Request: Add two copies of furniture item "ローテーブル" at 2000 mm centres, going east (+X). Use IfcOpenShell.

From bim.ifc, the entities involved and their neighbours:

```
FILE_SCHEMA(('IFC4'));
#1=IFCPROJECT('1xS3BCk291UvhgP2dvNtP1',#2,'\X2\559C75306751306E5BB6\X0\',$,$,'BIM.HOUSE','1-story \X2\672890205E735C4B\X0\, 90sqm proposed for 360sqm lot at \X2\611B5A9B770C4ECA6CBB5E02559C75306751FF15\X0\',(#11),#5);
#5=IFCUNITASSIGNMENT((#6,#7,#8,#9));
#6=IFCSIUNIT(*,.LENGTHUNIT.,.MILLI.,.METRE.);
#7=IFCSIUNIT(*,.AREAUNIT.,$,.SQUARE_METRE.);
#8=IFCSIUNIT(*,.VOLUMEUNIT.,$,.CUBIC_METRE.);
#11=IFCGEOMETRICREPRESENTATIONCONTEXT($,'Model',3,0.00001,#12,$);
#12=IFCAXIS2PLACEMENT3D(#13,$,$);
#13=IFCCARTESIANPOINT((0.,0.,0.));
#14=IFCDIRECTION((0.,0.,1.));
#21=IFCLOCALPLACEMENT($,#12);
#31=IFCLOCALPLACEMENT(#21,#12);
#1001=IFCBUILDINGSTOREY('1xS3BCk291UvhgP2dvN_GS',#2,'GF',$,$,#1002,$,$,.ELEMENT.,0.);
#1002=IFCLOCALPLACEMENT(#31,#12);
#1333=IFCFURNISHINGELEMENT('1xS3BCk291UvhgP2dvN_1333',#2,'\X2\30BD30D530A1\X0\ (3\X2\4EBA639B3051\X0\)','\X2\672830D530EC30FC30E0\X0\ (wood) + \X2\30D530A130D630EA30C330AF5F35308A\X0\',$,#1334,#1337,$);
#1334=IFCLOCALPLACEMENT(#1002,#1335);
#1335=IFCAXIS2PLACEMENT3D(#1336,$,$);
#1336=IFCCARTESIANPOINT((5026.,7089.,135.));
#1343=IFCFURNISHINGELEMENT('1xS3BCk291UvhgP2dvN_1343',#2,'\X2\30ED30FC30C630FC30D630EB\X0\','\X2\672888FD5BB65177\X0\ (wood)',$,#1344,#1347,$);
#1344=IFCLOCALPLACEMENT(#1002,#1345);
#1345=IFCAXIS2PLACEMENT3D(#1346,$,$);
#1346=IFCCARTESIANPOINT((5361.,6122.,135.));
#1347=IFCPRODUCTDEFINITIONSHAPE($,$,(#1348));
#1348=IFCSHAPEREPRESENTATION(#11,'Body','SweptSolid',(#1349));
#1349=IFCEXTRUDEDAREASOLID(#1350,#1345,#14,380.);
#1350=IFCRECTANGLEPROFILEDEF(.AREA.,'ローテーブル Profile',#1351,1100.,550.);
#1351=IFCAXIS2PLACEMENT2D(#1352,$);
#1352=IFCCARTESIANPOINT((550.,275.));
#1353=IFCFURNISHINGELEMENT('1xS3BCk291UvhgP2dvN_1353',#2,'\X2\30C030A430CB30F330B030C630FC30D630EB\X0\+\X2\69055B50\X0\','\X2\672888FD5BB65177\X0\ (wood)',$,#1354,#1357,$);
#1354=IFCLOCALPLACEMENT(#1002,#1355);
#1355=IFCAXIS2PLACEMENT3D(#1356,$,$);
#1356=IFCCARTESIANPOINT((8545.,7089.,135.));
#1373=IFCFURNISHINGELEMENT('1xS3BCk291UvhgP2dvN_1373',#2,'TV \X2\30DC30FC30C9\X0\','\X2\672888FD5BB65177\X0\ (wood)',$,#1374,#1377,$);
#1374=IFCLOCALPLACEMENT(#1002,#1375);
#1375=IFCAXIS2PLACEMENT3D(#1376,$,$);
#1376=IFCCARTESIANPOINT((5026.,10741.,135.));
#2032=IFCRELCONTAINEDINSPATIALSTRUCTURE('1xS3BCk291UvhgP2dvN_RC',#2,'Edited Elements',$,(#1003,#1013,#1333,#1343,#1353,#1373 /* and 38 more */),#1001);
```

```python
import numpy as np
import ifcopenshell
import ifcopenshell.api.geometry
import ifcopenshell.api.root
import ifcopenshell.util.element
import ifcopenshell.util.placement
import ifcopenshell.util.unit

model = ifcopenshell.open("bim.ifc")
unit_scale = ifcopenshell.util.unit.calculate_unit_scale(model)


def reuse_history(source, copy):
    """copy_class also copies each property set's owner history, people and application; keep the originals."""
    for rel in copy.IsDefinedBy:
        if rel.is_a("IfcRelDefinesByProperties") and (history := rel.RelatingPropertyDefinition.OwnerHistory):
            rel.RelatingPropertyDefinition.OwnerHistory = source.OwnerHistory
            ifcopenshell.util.element.remove_deep2(model, history)


source = model.by_guid("1xS3BCk291UvhgP2dvN_1343")
base = ifcopenshell.util.placement.get_local_placement(source.ObjectPlacement)
step = np.array([1.0, 0.0, 0.0]) * 2 / unit_scale

for i in range(1, 3):
    copy = ifcopenshell.api.root.copy_class(model, product=source)
    copy.Representation = ifcopenshell.util.element.copy_deep(
        model, source.Representation, exclude=["IfcGeometricRepresentationContext", "IfcRepresentationMap"]
    )
    reuse_history(source, copy)
    matrix = base.copy()
    matrix[:3, 3] += i * step
    print("added at", matrix[:3, 3].round(3) + 0.0)
    ifcopenshell.api.geometry.edit_object_placement(model, product=copy, matrix=matrix, is_si=False)

model.write("bim_edited.ifc")
```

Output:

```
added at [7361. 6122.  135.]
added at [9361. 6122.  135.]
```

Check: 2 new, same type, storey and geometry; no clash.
